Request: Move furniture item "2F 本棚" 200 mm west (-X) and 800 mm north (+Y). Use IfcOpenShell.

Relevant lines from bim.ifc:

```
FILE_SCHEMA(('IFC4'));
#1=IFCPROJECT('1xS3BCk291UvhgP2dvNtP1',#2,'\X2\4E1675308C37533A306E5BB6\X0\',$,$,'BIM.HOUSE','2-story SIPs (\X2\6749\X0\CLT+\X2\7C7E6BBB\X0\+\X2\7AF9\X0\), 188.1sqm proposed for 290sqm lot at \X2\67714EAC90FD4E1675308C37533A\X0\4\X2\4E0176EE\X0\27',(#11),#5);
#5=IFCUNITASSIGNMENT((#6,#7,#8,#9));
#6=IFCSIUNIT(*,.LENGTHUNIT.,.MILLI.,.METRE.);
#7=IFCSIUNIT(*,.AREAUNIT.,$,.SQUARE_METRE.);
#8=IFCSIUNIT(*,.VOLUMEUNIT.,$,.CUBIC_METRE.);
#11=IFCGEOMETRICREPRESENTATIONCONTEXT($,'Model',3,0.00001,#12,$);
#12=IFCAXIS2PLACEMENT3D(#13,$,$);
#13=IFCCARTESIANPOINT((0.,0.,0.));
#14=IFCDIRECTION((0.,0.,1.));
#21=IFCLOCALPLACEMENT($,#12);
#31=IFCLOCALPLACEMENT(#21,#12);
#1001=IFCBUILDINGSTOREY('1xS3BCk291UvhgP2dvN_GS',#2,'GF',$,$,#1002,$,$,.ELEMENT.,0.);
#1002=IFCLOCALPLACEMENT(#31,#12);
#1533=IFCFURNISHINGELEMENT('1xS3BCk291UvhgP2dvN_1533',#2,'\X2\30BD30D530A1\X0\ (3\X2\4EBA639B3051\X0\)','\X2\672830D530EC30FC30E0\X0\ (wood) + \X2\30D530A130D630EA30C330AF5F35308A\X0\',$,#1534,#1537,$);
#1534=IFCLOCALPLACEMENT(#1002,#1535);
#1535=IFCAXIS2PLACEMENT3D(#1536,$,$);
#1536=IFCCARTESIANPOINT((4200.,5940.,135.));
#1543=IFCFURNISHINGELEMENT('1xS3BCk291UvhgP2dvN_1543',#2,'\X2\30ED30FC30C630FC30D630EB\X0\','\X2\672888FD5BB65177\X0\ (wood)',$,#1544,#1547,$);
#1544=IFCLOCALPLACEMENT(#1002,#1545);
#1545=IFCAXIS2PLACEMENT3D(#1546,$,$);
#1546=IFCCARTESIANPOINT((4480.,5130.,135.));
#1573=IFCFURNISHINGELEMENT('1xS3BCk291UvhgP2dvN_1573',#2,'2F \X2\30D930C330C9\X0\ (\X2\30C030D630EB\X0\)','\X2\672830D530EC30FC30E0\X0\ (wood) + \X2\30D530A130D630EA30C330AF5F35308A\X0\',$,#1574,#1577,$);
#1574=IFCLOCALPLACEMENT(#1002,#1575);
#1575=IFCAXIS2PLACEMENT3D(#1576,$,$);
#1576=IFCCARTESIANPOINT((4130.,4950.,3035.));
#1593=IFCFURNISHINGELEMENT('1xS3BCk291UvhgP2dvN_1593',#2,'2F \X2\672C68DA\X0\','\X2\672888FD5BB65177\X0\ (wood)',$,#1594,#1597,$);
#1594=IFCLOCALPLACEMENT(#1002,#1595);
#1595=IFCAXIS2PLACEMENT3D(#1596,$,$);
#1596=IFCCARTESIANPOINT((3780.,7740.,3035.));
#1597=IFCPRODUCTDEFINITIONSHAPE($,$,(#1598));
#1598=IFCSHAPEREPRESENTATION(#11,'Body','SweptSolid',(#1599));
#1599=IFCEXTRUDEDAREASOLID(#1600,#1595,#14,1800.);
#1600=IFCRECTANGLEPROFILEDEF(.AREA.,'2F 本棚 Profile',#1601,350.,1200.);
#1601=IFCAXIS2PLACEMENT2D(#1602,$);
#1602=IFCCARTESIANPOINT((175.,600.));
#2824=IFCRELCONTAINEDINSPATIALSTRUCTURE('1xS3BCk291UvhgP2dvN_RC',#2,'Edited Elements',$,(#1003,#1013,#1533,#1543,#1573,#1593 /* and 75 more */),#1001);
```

```python
import ifcopenshell
import ifcopenshell.api.geometry
import ifcopenshell.util.placement

model = ifcopenshell.open("bim.ifc")

item = model.by_guid("1xS3BCk291UvhgP2dvN_1593")
matrix = ifcopenshell.util.placement.get_local_placement(item.ObjectPlacement)
matrix[0, 3] -= 200.0
matrix[1, 3] += 800.0
ifcopenshell.api.geometry.edit_object_placement(model, product=item, matrix=matrix, is_si=False)

print(ifcopenshell.util.placement.get_local_placement(item.ObjectPlacement).round(3) + 0.0)

model.write("bim_v2.ifc")
```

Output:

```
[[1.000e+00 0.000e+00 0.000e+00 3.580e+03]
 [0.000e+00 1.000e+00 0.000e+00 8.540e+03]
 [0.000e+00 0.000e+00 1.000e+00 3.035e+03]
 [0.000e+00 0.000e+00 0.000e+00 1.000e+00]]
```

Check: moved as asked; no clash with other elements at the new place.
